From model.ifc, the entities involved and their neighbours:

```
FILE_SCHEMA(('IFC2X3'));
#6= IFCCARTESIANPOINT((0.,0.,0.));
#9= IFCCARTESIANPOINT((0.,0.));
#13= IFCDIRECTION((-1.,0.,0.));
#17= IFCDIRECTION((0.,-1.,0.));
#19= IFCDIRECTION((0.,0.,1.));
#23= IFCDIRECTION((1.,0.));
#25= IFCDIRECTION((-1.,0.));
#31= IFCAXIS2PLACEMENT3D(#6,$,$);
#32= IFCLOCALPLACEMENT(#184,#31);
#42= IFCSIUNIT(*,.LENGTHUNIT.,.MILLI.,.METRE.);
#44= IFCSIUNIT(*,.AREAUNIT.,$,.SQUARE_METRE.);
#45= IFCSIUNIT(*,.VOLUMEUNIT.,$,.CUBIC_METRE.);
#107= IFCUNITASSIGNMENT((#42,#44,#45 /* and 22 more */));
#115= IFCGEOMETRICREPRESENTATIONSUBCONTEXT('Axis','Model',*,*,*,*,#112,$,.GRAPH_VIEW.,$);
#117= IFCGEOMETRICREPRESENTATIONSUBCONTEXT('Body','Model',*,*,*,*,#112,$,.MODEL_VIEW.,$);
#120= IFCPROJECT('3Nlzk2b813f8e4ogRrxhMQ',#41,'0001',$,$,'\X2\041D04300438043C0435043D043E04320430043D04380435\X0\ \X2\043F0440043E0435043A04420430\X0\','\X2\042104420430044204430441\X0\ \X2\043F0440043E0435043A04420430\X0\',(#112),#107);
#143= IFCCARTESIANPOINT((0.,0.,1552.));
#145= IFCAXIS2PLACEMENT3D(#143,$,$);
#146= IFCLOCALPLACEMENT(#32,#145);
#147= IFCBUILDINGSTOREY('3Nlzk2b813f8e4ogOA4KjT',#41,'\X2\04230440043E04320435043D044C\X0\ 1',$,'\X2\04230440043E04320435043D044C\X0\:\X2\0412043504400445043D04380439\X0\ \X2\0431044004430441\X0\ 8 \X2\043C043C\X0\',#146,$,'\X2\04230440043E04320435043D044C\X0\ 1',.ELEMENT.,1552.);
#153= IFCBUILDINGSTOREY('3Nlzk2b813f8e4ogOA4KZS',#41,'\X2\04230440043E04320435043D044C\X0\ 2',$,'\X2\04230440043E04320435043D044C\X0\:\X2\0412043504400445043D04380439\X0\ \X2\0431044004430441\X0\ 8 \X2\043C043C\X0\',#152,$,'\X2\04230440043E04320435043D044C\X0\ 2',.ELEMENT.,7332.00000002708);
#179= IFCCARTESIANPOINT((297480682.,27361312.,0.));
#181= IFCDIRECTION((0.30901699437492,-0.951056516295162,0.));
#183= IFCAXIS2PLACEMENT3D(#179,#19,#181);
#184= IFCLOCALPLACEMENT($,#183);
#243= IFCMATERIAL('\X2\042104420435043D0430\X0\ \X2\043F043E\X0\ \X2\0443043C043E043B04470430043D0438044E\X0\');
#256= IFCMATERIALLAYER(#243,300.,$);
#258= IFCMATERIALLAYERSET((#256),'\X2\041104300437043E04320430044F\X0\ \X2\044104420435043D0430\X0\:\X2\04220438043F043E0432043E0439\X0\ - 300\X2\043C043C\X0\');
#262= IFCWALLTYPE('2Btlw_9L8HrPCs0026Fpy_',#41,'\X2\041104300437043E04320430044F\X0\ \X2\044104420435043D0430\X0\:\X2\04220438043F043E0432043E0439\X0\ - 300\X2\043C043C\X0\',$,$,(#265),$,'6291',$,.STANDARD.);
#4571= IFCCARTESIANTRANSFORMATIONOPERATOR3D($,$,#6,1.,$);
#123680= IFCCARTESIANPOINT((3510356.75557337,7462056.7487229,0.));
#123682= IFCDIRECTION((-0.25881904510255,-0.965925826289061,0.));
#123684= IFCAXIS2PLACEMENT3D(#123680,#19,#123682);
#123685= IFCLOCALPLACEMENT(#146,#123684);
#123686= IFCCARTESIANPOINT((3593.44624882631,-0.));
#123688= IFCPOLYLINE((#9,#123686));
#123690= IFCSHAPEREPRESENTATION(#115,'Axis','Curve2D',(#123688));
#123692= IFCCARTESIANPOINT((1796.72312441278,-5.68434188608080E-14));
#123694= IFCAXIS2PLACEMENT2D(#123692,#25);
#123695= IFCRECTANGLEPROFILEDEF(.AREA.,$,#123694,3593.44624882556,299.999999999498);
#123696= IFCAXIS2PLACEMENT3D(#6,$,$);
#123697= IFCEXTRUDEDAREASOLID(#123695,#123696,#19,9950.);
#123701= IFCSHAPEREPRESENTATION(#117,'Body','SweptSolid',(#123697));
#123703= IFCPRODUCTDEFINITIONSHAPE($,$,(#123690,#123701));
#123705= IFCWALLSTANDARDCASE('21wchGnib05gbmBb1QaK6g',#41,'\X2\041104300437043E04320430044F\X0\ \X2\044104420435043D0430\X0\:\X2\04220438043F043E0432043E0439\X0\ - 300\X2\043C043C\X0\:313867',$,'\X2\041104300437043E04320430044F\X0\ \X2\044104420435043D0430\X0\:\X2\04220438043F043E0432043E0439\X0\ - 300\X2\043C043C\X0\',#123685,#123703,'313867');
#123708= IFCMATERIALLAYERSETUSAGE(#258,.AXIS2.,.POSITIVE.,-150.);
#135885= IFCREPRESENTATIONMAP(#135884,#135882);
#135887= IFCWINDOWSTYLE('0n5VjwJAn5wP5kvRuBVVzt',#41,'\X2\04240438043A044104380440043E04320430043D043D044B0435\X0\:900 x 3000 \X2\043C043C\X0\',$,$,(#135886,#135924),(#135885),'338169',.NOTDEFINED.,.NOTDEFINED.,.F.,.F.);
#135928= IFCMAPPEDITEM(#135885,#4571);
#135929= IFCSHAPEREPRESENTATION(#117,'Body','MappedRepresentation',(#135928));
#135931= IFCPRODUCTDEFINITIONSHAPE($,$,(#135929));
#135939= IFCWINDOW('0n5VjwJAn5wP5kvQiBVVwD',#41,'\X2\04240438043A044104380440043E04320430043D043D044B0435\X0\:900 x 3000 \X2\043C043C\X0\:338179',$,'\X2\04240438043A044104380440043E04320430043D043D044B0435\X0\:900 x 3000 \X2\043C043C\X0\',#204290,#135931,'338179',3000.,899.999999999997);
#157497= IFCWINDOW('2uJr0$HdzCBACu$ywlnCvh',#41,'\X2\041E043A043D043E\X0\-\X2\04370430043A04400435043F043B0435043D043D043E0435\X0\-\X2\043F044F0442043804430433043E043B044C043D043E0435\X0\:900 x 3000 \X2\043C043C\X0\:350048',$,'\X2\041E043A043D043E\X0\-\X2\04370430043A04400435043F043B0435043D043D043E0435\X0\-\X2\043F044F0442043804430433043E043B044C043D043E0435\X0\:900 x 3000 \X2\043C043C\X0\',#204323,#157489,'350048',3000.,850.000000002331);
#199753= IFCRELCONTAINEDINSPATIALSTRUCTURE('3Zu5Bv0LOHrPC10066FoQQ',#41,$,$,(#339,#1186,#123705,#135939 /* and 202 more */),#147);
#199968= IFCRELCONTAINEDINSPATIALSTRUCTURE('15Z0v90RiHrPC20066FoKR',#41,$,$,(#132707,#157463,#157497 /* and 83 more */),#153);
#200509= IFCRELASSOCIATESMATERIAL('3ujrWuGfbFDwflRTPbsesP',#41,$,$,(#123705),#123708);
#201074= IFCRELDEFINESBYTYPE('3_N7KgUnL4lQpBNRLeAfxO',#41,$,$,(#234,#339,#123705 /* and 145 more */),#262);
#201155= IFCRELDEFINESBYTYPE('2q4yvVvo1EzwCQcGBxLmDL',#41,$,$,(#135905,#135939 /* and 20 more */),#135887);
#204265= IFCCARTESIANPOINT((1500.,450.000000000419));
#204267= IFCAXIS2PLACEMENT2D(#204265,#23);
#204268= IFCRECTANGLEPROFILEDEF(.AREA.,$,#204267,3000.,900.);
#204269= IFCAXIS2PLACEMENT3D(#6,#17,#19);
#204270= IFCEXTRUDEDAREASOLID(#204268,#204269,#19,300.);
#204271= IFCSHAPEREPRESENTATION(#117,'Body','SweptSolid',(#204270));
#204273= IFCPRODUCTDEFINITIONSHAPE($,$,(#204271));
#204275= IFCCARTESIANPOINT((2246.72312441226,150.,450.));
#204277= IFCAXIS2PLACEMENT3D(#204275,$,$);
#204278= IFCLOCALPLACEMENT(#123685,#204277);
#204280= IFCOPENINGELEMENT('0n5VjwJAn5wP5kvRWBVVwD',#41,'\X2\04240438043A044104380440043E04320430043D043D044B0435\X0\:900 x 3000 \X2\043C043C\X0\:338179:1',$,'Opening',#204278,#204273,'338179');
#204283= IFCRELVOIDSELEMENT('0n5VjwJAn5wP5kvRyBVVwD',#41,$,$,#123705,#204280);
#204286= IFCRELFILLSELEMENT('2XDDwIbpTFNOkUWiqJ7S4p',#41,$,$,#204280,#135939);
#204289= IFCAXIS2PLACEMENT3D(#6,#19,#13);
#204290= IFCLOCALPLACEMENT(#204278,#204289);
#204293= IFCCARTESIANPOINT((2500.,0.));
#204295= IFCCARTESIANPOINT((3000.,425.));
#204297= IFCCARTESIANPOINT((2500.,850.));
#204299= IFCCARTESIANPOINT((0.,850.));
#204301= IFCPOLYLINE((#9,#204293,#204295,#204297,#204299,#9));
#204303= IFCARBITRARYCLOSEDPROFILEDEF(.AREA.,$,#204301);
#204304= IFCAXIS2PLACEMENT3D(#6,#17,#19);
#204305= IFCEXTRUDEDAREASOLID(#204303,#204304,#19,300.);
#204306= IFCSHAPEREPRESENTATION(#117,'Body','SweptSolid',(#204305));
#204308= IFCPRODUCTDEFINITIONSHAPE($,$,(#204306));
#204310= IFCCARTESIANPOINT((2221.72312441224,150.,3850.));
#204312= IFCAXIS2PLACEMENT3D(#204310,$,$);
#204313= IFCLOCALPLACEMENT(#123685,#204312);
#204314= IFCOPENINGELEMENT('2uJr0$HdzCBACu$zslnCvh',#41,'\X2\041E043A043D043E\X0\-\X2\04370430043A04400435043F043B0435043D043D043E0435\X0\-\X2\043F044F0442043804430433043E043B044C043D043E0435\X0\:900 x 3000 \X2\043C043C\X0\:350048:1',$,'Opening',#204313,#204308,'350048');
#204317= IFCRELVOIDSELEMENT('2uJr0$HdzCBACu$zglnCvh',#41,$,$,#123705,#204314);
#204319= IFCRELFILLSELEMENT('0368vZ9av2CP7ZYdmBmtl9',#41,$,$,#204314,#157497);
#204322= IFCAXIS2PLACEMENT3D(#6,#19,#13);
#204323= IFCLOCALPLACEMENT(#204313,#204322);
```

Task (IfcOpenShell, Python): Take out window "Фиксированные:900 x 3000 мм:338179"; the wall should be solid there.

```python
import ifcopenshell
import ifcopenshell.api.feature
import ifcopenshell.api.root
import ifcopenshell.geom
import ifcopenshell.util.shape

model = ifcopenshell.open("model.ifc")
settings = ifcopenshell.geom.settings()


def volume(element):
    """Net volume in cubic metres, openings subtracted."""
    shape = ifcopenshell.geom.create_shape(settings, element)
    return ifcopenshell.util.shape.get_volume(shape.geometry)


window = model.by_guid("0n5VjwJAn5wP5kvQiBVVwD")
opening = window.FillsVoids[0].RelatingOpeningElement
wall = opening.VoidsElements[0].RelatingBuildingElement
before = volume(wall)

ifcopenshell.api.root.remove_product(model, product=window)
ifcopenshell.api.feature.remove_feature(model, feature=opening)

after = volume(wall)

print(f"wall volume {before:.3f} -> {after:.3f} m3")

model.write("model_edited.ifc")
```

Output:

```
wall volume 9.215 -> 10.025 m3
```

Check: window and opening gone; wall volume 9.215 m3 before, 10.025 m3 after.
